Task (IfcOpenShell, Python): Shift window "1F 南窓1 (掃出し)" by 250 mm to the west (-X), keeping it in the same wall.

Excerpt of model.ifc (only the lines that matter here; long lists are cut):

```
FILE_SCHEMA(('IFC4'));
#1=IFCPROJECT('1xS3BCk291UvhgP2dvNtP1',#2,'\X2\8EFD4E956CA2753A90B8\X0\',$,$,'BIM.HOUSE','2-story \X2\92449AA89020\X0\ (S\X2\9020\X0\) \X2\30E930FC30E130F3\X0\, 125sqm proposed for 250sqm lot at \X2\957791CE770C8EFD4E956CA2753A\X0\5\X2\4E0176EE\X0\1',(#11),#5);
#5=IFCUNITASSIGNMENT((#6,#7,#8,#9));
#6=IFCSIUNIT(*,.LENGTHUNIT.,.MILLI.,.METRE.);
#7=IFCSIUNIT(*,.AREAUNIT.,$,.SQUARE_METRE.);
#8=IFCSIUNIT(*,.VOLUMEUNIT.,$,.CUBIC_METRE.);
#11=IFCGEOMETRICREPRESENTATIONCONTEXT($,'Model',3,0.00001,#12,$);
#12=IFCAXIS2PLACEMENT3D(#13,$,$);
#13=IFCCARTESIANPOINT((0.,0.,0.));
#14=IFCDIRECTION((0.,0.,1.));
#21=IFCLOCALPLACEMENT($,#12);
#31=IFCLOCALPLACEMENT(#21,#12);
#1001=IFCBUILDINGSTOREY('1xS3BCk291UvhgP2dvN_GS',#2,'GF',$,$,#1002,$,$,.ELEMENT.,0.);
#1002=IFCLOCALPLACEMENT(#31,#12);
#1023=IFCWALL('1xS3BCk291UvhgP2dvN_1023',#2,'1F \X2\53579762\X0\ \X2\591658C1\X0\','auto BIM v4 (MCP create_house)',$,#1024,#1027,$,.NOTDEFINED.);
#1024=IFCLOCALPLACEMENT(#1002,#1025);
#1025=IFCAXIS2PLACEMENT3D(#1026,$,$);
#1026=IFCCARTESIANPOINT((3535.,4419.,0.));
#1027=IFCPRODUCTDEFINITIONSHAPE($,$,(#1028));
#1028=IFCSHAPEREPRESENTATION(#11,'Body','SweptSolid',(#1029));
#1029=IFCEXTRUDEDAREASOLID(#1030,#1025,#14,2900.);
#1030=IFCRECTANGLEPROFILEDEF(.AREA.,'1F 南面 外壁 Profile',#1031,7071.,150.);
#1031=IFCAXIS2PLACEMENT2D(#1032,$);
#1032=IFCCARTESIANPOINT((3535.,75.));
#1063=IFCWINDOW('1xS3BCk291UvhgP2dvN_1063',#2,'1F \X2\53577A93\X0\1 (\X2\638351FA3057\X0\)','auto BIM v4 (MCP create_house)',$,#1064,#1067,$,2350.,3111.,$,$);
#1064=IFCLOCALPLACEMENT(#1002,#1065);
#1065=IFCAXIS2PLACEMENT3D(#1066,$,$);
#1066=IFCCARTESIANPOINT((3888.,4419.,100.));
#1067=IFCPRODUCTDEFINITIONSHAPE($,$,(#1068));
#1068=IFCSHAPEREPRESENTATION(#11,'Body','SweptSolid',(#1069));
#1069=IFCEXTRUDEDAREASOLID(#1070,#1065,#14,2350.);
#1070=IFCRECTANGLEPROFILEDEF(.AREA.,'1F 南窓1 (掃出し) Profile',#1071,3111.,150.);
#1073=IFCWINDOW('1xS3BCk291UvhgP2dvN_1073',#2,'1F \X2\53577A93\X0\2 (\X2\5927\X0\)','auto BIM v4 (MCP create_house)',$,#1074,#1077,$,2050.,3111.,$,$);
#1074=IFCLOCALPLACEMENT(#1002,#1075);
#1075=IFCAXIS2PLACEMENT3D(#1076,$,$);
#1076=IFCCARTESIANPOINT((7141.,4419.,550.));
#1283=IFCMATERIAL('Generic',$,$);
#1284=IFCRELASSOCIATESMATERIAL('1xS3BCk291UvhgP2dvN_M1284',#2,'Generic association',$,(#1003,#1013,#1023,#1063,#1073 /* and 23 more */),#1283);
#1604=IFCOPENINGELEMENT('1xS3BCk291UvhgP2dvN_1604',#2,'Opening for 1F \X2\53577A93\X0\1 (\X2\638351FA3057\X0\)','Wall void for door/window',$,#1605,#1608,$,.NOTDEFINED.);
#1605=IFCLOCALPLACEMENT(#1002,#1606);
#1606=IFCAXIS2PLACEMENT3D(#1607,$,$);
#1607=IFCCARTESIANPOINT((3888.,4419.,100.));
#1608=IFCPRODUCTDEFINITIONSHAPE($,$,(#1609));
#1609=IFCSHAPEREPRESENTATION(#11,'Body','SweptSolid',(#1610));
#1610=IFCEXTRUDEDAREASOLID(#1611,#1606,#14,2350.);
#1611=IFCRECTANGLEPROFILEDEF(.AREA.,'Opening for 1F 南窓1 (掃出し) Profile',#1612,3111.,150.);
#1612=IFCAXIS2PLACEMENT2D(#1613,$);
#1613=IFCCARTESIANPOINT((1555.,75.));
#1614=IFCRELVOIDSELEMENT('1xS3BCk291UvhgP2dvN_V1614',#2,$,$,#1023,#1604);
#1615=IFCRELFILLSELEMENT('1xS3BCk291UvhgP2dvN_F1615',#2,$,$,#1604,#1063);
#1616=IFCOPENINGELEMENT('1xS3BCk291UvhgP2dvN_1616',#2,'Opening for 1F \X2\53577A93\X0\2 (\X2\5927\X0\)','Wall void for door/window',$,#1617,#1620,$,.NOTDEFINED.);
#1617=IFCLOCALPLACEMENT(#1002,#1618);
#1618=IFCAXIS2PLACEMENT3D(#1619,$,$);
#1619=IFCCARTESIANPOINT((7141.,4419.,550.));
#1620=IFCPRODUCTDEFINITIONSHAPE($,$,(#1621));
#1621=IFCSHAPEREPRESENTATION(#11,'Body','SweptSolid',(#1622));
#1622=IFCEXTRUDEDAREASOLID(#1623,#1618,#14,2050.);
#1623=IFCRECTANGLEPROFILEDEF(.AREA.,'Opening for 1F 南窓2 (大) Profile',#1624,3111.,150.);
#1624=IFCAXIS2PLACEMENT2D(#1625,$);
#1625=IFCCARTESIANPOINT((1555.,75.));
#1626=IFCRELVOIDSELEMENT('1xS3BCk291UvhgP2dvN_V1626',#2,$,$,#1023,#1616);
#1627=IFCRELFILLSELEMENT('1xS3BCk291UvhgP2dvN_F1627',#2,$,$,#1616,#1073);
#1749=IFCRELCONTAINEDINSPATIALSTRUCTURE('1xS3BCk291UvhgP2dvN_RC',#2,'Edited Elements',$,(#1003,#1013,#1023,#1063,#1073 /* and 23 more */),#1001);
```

```python
import ifcopenshell
import ifcopenshell.api.geometry
import ifcopenshell.util.placement
import ifcopenshell.util.unit

model = ifcopenshell.open("model.ifc")
unit_scale = ifcopenshell.util.unit.calculate_unit_scale(model)

window = model.by_guid("1xS3BCk291UvhgP2dvN_1063")
opening = window.FillsVoids[0].RelatingOpeningElement
wall = opening.VoidsElements[0].RelatingBuildingElement

wall_matrix = ifcopenshell.util.placement.get_local_placement(wall.ObjectPlacement)
shift = wall_matrix[:3, 0] * -0.25 / unit_scale
before = ifcopenshell.util.placement.get_local_placement(window.ObjectPlacement)[:3, 3].copy()

# The window is not placed relative to its opening, so move both.
for product in (opening, window):
    matrix = ifcopenshell.util.placement.get_local_placement(product.ObjectPlacement)
    matrix[:3, 3] += shift
    ifcopenshell.api.geometry.edit_object_placement(model, product=product, matrix=matrix, is_si=False)

after = ifcopenshell.util.placement.get_local_placement(window.ObjectPlacement)[:3, 3]
print("window moved by", (after - before).round(3) + 0.0)

model.write("model_v2.ifc")
```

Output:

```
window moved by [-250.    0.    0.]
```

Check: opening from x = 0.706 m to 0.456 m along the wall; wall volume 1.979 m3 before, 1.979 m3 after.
